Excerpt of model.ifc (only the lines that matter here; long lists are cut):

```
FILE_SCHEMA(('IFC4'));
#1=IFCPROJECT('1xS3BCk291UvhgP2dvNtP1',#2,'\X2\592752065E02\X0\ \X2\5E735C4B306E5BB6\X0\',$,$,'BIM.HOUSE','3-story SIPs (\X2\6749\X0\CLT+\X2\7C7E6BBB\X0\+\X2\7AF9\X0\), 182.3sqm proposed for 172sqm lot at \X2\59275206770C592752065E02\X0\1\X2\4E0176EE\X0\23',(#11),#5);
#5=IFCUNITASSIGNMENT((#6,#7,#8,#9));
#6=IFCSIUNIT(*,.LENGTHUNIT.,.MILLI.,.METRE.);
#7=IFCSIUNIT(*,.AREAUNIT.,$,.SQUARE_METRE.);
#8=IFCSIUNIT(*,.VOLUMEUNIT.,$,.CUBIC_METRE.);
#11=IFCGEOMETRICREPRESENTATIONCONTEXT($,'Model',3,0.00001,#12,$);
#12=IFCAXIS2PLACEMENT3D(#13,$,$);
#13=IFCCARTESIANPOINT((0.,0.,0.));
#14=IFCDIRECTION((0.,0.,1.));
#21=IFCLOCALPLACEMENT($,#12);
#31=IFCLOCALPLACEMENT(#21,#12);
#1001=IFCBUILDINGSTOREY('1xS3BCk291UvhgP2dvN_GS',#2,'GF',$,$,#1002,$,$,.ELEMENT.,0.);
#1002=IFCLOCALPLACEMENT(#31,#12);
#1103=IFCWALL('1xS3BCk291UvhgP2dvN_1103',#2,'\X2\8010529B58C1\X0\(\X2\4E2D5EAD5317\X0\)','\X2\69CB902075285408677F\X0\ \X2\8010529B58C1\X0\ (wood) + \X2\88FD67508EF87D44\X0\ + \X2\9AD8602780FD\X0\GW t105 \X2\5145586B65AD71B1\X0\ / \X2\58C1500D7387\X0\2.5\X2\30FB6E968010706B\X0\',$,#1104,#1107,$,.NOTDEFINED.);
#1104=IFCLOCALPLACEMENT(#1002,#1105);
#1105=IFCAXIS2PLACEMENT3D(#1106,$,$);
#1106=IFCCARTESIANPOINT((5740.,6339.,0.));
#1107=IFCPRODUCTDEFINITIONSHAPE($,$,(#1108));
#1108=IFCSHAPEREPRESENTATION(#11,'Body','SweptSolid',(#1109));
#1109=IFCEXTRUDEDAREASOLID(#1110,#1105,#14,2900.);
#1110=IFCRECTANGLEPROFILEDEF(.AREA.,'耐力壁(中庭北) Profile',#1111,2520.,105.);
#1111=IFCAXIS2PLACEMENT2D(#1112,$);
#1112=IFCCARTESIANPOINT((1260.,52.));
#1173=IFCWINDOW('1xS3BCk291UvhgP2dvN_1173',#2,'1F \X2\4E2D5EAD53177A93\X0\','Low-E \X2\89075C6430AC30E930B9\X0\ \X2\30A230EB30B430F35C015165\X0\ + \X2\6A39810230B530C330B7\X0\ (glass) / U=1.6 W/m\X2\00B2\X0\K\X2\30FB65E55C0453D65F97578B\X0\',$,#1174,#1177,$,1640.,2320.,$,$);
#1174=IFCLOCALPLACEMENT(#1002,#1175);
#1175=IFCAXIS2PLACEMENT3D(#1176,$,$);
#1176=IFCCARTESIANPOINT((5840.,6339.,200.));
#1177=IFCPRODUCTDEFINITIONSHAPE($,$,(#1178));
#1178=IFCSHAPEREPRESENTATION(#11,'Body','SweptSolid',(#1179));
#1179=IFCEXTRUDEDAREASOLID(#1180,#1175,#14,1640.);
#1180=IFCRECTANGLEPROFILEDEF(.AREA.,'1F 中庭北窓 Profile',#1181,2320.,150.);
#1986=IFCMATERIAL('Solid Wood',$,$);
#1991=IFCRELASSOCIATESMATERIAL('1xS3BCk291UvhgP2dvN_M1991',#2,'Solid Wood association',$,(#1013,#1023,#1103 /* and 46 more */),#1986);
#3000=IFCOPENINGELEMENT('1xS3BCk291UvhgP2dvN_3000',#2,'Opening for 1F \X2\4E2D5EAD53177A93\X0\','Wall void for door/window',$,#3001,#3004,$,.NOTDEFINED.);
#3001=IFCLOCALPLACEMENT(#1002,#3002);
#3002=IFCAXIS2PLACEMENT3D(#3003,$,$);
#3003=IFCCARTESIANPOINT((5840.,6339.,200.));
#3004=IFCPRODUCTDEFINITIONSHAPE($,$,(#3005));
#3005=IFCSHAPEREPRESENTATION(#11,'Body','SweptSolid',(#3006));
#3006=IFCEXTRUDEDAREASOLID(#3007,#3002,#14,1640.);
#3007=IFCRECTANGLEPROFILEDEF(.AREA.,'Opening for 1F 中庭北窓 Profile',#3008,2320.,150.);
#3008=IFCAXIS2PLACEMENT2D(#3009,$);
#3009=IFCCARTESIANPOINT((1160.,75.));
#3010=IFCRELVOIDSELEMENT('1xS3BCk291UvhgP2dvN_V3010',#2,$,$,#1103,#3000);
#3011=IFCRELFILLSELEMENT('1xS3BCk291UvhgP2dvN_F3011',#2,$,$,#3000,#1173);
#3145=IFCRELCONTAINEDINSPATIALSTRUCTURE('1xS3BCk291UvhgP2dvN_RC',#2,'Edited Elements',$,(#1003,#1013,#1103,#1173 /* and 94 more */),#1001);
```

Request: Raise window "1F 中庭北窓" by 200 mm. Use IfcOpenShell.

```python
import numpy as np
import ifcopenshell
import ifcopenshell.api.geometry
import ifcopenshell.util.placement
import ifcopenshell.util.unit

model = ifcopenshell.open("model.ifc")
unit_scale = ifcopenshell.util.unit.calculate_unit_scale(model)

window = model.by_guid("1xS3BCk291UvhgP2dvN_1173")
opening = window.FillsVoids[0].RelatingOpeningElement
dz = 200.0

shift = np.array([0.0, 0.0, dz])
# The window is not placed relative to its opening, so move both.
for product in (opening, window):
    matrix = ifcopenshell.util.placement.get_local_placement(product.ObjectPlacement)
    matrix[:3, 3] += shift
    ifcopenshell.api.geometry.edit_object_placement(model, product=product, matrix=matrix, is_si=False)

print(f"moved by {dz * unit_scale:+.3f} m")

model.write("model_edited.ifc")
```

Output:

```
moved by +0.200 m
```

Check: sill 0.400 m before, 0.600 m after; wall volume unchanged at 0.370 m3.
